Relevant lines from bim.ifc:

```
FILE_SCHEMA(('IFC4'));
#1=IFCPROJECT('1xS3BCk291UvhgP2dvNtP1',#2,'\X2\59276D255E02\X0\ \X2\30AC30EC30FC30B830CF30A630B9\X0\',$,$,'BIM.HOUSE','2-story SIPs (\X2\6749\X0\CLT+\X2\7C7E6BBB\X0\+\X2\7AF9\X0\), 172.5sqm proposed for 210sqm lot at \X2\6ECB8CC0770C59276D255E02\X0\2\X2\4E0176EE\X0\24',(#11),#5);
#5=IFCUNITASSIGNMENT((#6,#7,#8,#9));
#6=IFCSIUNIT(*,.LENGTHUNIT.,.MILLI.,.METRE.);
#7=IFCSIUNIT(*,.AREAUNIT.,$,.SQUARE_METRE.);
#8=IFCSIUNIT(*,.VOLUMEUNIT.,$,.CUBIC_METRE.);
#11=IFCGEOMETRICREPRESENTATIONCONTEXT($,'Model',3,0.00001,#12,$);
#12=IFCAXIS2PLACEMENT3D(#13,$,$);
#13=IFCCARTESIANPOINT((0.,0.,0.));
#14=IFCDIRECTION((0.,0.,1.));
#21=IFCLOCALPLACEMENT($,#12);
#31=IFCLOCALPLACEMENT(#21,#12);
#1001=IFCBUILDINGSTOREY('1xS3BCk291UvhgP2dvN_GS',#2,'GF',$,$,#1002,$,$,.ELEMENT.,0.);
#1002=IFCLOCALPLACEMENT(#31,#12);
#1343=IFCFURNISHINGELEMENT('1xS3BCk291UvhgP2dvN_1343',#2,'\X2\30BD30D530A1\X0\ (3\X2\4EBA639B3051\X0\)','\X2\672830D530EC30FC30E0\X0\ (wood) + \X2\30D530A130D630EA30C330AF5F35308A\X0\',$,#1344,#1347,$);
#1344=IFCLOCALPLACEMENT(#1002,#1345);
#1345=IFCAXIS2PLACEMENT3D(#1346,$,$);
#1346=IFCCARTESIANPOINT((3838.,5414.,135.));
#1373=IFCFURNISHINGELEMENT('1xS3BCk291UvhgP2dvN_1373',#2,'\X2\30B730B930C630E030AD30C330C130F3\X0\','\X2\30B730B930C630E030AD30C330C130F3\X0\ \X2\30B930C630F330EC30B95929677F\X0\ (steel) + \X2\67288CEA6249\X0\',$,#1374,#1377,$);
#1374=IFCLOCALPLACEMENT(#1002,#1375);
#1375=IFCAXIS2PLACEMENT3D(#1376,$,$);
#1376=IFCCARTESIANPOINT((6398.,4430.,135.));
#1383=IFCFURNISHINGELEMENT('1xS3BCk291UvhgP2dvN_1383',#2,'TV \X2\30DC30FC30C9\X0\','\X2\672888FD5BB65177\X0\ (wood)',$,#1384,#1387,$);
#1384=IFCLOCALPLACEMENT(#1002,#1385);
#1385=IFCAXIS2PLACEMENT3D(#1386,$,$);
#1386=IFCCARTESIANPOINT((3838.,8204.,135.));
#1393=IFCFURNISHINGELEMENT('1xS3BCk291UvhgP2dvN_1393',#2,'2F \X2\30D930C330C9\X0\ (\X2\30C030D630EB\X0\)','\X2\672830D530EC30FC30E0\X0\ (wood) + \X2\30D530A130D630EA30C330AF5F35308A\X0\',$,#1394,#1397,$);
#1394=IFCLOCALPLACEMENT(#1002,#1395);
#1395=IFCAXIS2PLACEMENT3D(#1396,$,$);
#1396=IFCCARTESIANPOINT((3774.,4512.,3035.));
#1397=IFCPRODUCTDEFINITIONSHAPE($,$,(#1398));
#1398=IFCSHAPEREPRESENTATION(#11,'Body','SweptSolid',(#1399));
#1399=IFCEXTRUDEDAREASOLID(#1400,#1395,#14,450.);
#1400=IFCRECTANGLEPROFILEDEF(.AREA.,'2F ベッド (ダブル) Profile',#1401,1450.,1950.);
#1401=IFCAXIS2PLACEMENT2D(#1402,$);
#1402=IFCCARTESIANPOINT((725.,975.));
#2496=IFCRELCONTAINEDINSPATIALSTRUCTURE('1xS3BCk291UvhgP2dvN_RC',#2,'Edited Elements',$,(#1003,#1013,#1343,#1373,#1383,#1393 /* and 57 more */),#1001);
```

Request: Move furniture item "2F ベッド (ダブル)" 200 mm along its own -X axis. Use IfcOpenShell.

```python
import ifcopenshell
import ifcopenshell.api.geometry
import ifcopenshell.util.placement
import ifcopenshell.util.unit

model = ifcopenshell.open("bim.ifc")
unit_scale = ifcopenshell.util.unit.calculate_unit_scale(model)

item = model.by_id(1393)
matrix = ifcopenshell.util.placement.get_local_placement(item.ObjectPlacement)
matrix[:3, 3] -= matrix[:3, 0] * 0.2 / unit_scale
ifcopenshell.api.geometry.edit_object_placement(model, product=item, matrix=matrix, is_si=False)

print(ifcopenshell.util.placement.get_local_placement(item.ObjectPlacement).round(3) + 0.0)

model.write("bim_updated.ifc")
```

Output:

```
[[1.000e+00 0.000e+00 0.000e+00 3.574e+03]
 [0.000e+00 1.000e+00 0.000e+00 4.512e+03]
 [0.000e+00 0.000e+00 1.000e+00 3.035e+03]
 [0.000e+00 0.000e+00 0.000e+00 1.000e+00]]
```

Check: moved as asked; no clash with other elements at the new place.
